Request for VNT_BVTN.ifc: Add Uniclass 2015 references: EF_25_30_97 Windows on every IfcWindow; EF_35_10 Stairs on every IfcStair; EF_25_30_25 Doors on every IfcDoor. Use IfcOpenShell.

First a look at what the model holds.

```python
import ifcopenshell

model = ifcopenshell.open("VNT_BVTN.ifc")
print(model.schema)
print("classifications:", [c.Name for c in model.by_type("IfcClassification")])
for ifc_class in ("IfcDoor", "IfcRoof", "IfcStair", "IfcWall", "IfcWindow"):
    print(ifc_class, len(model.by_type(ifc_class)))
```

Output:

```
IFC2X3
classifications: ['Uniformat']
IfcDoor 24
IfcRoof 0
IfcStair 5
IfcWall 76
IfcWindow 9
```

```python
import ifcopenshell
import ifcopenshell.api.classification

model = ifcopenshell.open("VNT_BVTN.ifc")

# IFC2X3 requires Source and Edition and has no link from the project to the system.
system = model.create_entity("IfcClassification", Source="NBS", Edition="2015", Name="Uniclass 2015")

codes = {
    "IfcWindow": ("EF_25_30_97", "Windows"),
    "IfcStair": ("EF_35_10", "Stairs"),
    "IfcDoor": ("EF_25_30_25", "Doors"),
}
for ifc_class, (code, name) in codes.items():
    products = model.by_type(ifc_class)
    ifcopenshell.api.classification.add_reference(
        model, products=products, classification=system, identification=code, name=name
    )
    print(code, len(products))

model.write("VNT_BVTN_v2.ifc")
```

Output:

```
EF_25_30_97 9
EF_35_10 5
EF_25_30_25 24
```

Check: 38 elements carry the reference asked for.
